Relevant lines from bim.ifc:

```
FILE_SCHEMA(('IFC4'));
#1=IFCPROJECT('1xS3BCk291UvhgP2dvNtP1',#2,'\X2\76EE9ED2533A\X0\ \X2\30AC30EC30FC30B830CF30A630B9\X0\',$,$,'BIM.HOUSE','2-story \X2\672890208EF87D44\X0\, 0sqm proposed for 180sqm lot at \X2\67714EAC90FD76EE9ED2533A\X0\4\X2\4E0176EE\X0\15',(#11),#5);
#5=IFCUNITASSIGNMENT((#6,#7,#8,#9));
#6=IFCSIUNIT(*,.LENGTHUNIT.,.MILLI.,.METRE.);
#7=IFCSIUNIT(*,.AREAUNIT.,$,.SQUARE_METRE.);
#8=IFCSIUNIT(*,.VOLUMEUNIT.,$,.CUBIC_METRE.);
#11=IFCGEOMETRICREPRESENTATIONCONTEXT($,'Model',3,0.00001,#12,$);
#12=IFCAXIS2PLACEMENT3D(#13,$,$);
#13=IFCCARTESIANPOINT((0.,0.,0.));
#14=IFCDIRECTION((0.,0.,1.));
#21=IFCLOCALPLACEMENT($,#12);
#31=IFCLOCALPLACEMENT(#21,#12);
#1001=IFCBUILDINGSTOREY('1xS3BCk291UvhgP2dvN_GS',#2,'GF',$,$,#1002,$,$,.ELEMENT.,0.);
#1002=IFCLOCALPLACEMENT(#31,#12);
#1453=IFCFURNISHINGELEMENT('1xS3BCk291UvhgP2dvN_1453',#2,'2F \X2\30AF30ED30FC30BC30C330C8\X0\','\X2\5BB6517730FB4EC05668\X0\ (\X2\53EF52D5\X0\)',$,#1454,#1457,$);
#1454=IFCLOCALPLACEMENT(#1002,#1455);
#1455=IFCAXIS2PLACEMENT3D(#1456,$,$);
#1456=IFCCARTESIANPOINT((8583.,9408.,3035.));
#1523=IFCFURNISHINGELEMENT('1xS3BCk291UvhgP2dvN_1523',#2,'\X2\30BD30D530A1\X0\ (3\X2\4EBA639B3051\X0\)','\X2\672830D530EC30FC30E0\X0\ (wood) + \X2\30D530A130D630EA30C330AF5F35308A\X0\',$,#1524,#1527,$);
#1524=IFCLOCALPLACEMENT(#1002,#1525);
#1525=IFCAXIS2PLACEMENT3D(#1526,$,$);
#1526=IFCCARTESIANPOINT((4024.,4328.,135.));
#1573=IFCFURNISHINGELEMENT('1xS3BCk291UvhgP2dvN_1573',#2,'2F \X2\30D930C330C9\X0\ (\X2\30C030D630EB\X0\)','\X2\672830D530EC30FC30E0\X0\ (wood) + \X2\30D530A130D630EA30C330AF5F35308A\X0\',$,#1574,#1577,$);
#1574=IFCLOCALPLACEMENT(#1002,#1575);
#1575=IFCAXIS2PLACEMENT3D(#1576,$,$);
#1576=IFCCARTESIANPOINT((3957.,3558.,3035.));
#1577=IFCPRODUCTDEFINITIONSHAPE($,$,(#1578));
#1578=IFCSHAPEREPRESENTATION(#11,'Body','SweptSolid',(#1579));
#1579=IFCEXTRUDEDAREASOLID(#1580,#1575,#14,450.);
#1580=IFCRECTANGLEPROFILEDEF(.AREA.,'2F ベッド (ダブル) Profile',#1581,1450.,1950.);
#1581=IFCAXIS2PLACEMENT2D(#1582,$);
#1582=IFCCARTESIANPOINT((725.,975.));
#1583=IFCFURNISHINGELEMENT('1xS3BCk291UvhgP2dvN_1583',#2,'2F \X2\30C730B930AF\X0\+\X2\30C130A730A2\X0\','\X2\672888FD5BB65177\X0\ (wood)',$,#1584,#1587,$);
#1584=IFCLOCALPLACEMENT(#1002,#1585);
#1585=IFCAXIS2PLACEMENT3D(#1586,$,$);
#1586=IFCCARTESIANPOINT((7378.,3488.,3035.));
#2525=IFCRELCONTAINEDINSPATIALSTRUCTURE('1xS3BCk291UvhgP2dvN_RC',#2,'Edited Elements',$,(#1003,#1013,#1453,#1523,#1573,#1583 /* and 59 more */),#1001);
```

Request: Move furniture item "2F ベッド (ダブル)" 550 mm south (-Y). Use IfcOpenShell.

```python
import ifcopenshell
import ifcopenshell.api.geometry
import ifcopenshell.util.placement
import ifcopenshell.util.unit

model = ifcopenshell.open("bim.ifc")
unit_scale = ifcopenshell.util.unit.calculate_unit_scale(model)

item = model.by_guid("1xS3BCk291UvhgP2dvN_1573")
matrix = ifcopenshell.util.placement.get_local_placement(item.ObjectPlacement)
matrix[1, 3] -= 0.55 / unit_scale
ifcopenshell.api.geometry.edit_object_placement(model, product=item, matrix=matrix, is_si=False)

print(ifcopenshell.util.placement.get_local_placement(item.ObjectPlacement).round(3) + 0.0)

model.write("bim_updated.ifc")
```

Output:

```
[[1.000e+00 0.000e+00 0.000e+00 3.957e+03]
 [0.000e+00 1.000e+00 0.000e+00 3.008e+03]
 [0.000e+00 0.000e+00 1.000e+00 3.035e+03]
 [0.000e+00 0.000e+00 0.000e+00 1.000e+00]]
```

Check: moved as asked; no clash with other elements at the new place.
